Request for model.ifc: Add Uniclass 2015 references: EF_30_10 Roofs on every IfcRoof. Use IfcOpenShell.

First a look at what the model holds.

```python
import ifcopenshell

model = ifcopenshell.open("model.ifc")
print(model.schema)
print("classifications:", [c.Name for c in model.by_type("IfcClassification")])
for ifc_class in ("IfcDoor", "IfcRoof", "IfcStair", "IfcWall", "IfcWindow"):
    print(ifc_class, len(model.by_type(ifc_class)))
```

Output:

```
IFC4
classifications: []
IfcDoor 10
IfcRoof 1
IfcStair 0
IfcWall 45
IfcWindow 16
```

```python
import ifcopenshell
import ifcopenshell.api.classification

model = ifcopenshell.open("model.ifc")

system = ifcopenshell.api.classification.add_classification(model, classification="Uniclass 2015")

codes = {
    "IfcRoof": ("EF_30_10", "Roofs"),
}
for ifc_class, (code, name) in codes.items():
    products = model.by_type(ifc_class)
    ifcopenshell.api.classification.add_reference(
        model, products=products, classification=system, identification=code, name=name
    )
    print(code, len(products))

model.write("model_edited.ifc")
```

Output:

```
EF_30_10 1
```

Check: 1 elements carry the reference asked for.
